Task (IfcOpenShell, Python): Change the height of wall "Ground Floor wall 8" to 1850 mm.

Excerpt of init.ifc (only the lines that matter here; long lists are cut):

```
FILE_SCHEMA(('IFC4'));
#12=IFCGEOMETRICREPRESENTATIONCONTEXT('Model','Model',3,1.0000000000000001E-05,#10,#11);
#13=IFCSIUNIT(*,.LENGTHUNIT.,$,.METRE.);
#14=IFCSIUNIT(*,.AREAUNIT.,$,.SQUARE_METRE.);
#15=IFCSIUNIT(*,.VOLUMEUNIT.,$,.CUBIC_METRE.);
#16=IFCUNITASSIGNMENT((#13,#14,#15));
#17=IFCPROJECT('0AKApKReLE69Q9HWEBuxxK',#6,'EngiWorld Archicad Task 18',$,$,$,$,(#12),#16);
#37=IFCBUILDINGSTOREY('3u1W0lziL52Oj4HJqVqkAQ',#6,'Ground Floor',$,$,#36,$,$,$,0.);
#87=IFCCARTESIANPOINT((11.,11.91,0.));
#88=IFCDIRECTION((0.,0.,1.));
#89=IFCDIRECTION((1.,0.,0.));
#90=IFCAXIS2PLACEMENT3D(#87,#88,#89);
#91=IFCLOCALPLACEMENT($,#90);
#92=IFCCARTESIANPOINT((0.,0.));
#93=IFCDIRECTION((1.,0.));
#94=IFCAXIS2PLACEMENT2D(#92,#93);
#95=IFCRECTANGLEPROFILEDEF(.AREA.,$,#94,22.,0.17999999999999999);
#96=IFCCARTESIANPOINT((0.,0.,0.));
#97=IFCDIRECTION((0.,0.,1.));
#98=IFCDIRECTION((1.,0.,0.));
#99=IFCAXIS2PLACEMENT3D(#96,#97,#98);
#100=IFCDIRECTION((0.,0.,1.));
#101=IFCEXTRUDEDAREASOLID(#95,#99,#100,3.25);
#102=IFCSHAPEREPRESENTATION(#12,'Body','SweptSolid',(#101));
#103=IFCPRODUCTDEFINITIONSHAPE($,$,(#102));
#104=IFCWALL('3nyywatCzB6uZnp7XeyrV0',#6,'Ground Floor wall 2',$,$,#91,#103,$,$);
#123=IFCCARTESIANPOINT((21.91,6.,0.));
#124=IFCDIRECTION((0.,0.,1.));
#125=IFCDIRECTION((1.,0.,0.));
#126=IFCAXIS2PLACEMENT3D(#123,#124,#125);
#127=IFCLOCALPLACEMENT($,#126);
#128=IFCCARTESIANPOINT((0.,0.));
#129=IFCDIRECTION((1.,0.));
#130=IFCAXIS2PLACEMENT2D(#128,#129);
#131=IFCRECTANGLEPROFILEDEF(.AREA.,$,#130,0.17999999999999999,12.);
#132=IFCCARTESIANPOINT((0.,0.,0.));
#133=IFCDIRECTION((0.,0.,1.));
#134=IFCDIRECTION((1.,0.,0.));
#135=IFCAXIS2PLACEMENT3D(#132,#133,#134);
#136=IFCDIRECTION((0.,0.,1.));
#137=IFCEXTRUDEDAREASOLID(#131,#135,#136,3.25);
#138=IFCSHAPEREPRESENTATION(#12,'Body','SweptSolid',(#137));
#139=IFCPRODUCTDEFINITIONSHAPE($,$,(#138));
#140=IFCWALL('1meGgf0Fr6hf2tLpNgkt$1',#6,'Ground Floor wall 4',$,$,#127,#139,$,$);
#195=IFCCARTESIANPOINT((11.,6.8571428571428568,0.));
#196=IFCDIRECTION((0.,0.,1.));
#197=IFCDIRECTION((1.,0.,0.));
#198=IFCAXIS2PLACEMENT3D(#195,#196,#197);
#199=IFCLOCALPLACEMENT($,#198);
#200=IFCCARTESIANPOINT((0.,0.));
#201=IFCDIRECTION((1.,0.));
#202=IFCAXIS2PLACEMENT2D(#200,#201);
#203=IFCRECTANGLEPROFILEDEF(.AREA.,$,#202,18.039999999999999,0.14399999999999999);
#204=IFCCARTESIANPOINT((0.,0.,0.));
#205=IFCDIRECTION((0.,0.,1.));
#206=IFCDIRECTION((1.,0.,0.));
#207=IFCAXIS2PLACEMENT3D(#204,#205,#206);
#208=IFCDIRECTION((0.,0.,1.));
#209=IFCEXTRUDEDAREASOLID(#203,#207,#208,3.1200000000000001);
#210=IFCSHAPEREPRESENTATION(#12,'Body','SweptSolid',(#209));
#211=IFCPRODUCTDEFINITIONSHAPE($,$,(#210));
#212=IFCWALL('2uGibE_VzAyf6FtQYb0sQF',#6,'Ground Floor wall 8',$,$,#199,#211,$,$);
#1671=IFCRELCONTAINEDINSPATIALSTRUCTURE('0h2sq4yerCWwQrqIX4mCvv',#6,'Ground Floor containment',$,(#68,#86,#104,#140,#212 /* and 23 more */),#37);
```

```python
import ifcopenshell
import ifcopenshell.geom
import ifcopenshell.util.shape
import ifcopenshell.util.unit

model = ifcopenshell.open("init.ifc")
unit_scale = ifcopenshell.util.unit.calculate_unit_scale(model)
settings = ifcopenshell.geom.settings()


def volume(element):
    """Net volume in cubic metres, openings subtracted."""
    shape = ifcopenshell.geom.create_shape(settings, element)
    return ifcopenshell.util.shape.get_volume(shape.geometry)


wall = model.by_guid("2uGibE_VzAyf6FtQYb0sQF")
before = volume(wall)

body = next(r for r in wall.Representation.Representations if r.RepresentationIdentifier == "Body")
solid = body.Items[0]
old_height = solid.Depth
solid.Depth = 1.85 / unit_scale
after = volume(wall)

print(f"height {old_height:g} -> {solid.Depth:g}, volume {before:.3f} -> {after:.3f} m3")

model.write("init_edited.ifc")
```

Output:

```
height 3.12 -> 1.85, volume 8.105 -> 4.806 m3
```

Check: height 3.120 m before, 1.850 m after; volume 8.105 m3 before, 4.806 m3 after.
